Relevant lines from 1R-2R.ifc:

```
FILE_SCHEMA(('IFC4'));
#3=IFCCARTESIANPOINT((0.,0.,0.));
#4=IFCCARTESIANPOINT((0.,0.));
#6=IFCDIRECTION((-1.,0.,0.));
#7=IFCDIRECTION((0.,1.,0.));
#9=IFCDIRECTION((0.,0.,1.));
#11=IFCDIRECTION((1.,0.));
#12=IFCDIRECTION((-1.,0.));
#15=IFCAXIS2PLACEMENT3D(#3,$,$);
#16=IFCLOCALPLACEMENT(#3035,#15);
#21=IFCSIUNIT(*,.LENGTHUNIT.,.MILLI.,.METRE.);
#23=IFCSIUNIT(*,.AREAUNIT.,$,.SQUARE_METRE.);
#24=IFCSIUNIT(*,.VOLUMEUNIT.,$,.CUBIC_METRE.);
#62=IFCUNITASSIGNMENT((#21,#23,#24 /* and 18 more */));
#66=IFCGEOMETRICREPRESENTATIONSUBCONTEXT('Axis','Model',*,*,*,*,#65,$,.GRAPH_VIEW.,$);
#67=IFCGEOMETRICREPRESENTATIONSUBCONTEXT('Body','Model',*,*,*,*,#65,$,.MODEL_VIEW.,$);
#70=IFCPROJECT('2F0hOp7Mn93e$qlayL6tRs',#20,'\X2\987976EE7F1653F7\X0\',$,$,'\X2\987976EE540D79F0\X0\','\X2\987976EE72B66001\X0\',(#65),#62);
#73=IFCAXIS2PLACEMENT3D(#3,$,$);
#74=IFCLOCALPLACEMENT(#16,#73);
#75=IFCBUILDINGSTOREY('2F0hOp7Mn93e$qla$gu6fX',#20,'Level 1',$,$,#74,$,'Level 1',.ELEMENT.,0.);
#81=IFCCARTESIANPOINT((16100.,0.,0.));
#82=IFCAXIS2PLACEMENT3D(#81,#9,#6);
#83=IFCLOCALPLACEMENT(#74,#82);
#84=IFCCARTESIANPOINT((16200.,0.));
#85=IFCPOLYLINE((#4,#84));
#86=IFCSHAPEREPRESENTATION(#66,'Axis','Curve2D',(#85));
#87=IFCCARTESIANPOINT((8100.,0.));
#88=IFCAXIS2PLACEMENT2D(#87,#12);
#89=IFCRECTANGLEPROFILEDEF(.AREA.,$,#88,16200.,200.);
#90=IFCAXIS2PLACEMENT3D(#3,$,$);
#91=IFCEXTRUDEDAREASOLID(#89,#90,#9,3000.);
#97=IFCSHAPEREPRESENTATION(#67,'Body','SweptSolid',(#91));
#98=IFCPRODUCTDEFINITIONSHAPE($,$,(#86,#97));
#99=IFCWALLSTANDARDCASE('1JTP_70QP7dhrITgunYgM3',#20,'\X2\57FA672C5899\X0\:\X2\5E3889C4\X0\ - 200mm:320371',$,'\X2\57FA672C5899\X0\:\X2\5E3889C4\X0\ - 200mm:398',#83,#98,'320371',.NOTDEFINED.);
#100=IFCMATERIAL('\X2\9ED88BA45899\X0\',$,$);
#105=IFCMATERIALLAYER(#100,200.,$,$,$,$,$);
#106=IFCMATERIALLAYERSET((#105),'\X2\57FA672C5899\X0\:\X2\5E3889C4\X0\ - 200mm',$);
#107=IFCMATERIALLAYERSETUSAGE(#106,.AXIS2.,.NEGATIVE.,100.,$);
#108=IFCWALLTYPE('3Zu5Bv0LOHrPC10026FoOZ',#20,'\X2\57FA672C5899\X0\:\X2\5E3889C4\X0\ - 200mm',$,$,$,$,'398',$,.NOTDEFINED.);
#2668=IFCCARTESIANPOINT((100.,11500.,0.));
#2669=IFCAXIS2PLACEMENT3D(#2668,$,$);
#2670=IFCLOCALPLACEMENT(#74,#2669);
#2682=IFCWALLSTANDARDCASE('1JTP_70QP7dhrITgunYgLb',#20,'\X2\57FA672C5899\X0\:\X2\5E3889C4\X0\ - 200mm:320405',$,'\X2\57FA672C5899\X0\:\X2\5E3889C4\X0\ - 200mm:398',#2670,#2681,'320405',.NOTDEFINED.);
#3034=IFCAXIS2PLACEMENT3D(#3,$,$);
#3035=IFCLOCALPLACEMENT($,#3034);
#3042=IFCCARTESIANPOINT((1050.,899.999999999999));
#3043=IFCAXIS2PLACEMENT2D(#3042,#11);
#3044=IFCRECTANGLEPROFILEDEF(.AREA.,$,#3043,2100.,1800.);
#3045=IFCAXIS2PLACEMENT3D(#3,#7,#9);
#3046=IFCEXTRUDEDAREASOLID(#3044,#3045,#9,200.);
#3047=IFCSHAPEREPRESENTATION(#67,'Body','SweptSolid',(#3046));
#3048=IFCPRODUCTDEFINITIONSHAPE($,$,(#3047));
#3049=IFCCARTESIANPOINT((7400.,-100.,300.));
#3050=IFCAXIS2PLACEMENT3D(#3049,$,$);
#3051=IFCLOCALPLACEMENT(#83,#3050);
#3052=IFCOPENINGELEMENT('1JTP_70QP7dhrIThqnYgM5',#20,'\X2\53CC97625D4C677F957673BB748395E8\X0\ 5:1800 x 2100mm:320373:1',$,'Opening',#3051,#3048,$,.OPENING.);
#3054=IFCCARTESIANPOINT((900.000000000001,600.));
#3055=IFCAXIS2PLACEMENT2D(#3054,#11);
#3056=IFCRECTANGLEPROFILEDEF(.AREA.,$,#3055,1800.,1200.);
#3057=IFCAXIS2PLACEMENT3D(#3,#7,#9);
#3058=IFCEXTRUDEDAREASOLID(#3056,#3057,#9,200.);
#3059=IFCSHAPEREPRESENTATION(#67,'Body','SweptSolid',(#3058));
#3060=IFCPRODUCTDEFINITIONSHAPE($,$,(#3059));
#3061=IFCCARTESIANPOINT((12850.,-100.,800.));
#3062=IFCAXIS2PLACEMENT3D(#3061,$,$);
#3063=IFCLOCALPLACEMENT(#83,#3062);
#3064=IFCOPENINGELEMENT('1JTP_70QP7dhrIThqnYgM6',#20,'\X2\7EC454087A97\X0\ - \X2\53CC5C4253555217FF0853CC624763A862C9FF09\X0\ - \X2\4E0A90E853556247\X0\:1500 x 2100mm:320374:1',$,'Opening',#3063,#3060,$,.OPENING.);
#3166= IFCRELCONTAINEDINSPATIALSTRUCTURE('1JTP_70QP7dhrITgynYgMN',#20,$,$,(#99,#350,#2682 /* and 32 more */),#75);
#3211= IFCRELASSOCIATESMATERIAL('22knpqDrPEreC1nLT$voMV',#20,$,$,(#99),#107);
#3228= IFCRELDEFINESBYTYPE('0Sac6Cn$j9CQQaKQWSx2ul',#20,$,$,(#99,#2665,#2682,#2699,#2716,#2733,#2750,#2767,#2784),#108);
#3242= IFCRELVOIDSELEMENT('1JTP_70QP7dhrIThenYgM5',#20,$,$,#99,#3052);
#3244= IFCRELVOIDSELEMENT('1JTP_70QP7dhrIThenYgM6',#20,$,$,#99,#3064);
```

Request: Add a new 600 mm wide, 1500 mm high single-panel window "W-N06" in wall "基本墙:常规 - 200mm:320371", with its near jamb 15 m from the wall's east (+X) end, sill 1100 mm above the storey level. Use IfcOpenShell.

```python
import numpy as np
import ifcopenshell
import ifcopenshell.api.feature
import ifcopenshell.api.geometry
import ifcopenshell.api.root
import ifcopenshell.api.spatial
import ifcopenshell.geom
import ifcopenshell.util.element
import ifcopenshell.util.placement
import ifcopenshell.util.representation
import ifcopenshell.util.shape
import ifcopenshell.util.unit

model = ifcopenshell.open("1R-2R.ifc")
unit_scale = ifcopenshell.util.unit.calculate_unit_scale(model)
settings = ifcopenshell.geom.settings()


def volume(element):
    """Net volume in cubic metres, openings subtracted."""
    shape = ifcopenshell.geom.create_shape(settings, element)
    return ifcopenshell.util.shape.get_volume(shape.geometry)


wall = model.by_guid("1JTP_70QP7dhrITgunYgM3")
storey = ifcopenshell.util.element.get_container(wall, ifc_class="IfcBuildingStorey")
context = ifcopenshell.util.representation.get_context(model, "Model", "Body", "MODEL_VIEW")
before = volume(wall)

width, height, from_end, sill = 0.6, 1.5, 15, 1.1  # metres

# The wall runs along its own X axis, and the end named is its -X end.
wall_shape = ifcopenshell.geom.create_shape(settings, wall)
x, y, z = ifcopenshell.util.shape.get_vertices(wall_shape.geometry).T
start = x.min() + from_end
face, thickness = float(y.min()), float(y.max() - y.min())
wall_matrix = ifcopenshell.util.placement.get_local_placement(wall.ObjectPlacement)
level = ifcopenshell.util.placement.get_local_placement(storey.ObjectPlacement)[2, 3]


def in_wall(x, y):
    """Placement at x, y metres in the wall's axes, at sill height."""
    matrix = wall_matrix.copy()
    matrix[:, 3] = wall_matrix @ np.array([x / unit_scale, y / unit_scale, 0.0, 1.0])
    matrix[2, 3] = level + sill / unit_scale
    return matrix


# Opening: a box that overshoots both wall faces by 50 mm.
opening = ifcopenshell.api.root.create_entity(model, ifc_class="IfcOpeningElement", predefined_type="OPENING")
box = ifcopenshell.api.geometry.add_wall_representation(
    model, context=context, length=width, height=height, thickness=thickness + 0.1
)
ifcopenshell.api.geometry.assign_representation(model, product=opening, representation=box)
ifcopenshell.api.geometry.edit_object_placement(model, product=opening, matrix=in_wall(start, face - 0.05), is_si=False)
ifcopenshell.api.feature.add_feature(model, feature=opening, element=wall)

window = ifcopenshell.api.root.create_entity(model, ifc_class="IfcWindow", name="W-N06", predefined_type="WINDOW")
window.OverallWidth, window.OverallHeight = width / unit_scale, height / unit_scale
window.PartitioningType = "SINGLE_PANEL"
body = ifcopenshell.api.geometry.add_window_representation(
    model,
    context=context,
    overall_width=window.OverallWidth,
    overall_height=window.OverallHeight,
    partition_type="SINGLE_PANEL",
)
ifcopenshell.api.geometry.assign_representation(model, product=window, representation=body)
ifcopenshell.api.spatial.assign_container(model, products=[window], relating_structure=storey)
ifcopenshell.api.feature.add_filling(model, opening=opening, element=window)

# Centre the window in the wall's thickness.
ifcopenshell.api.geometry.edit_object_placement(model, product=window, matrix=in_wall(start, face), is_si=False)
window_shape = ifcopenshell.geom.create_shape(settings, window)
depth = ifcopenshell.util.shape.get_vertices(window_shape.geometry)[:, 1]
offset = face + thickness / 2 - (depth.min() + depth.max()) / 2
ifcopenshell.api.geometry.edit_object_placement(model, product=window, matrix=in_wall(start, offset), is_si=False)

after = volume(wall)

print(f"wall volume {before:.3f} -> {after:.3f} m3")

model.write("1R-2R_updated.ifc")
```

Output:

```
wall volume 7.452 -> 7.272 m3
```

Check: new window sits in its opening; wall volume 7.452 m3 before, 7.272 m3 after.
